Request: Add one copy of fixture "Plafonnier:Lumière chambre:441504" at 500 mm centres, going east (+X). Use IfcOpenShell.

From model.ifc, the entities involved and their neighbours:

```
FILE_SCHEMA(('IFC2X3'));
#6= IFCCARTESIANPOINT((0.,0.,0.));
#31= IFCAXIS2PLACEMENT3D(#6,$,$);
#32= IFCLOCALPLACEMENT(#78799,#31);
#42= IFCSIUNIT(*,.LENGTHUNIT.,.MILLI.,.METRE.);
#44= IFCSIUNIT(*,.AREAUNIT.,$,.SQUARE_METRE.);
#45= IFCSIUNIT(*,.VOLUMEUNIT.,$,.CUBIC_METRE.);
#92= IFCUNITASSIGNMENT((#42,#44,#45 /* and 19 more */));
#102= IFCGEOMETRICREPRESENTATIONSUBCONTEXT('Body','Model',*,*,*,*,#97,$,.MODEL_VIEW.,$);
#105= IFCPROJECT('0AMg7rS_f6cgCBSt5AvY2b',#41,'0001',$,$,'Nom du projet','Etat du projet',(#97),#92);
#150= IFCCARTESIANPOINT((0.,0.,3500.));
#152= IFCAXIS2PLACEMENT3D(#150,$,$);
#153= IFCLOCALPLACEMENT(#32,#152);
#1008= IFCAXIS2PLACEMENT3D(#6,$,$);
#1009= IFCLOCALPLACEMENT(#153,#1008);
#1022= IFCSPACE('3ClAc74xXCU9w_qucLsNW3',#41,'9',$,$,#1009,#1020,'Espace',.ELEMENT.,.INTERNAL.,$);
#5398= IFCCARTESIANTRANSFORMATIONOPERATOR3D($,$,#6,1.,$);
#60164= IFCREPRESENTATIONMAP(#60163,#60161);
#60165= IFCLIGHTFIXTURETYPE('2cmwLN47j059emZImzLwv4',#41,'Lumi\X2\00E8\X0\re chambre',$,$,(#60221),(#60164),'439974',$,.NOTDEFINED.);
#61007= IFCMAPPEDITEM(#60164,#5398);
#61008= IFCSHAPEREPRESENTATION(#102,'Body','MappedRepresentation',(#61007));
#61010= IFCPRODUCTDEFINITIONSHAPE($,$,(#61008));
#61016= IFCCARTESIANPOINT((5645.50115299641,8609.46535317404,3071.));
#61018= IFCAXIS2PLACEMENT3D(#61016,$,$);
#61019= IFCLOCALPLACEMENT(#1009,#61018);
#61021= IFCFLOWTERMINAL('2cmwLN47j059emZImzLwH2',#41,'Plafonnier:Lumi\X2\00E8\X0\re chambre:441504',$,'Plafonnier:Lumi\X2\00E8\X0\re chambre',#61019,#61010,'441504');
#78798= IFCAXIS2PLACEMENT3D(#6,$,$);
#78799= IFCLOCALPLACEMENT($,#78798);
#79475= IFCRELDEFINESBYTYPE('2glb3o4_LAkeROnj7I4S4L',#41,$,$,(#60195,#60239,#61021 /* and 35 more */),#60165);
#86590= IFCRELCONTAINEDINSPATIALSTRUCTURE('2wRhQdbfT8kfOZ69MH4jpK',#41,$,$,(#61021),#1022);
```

```python
import numpy as np
import ifcopenshell
import ifcopenshell.api.geometry
import ifcopenshell.api.root
import ifcopenshell.util.element
import ifcopenshell.util.placement

model = ifcopenshell.open("model.ifc")


def reuse_history(source, copy):
    """copy_class also copies each property set's owner history, people and application; keep the originals."""
    for rel in copy.IsDefinedBy:
        if rel.is_a("IfcRelDefinesByProperties") and (history := rel.RelatingPropertyDefinition.OwnerHistory):
            rel.RelatingPropertyDefinition.OwnerHistory = source.OwnerHistory
            ifcopenshell.util.element.remove_deep2(model, history)


source = model.by_guid("2cmwLN47j059emZImzLwH2")
base = ifcopenshell.util.placement.get_local_placement(source.ObjectPlacement)
step = np.array([1.0, 0.0, 0.0]) * 500.0

for i in range(1, 2):
    copy = ifcopenshell.api.root.copy_class(model, product=source)
    copy.Representation = ifcopenshell.util.element.copy_deep(
        model, source.Representation, exclude=["IfcGeometricRepresentationContext", "IfcRepresentationMap"]
    )
    copy.Name = "Plafonnier:Lumière chambre"
    copy.Tag = None
    reuse_history(source, copy)
    matrix = base.copy()
    matrix[:3, 3] += i * step
    print("added at", matrix[:3, 3].round(3) + 0.0)
    ifcopenshell.api.geometry.edit_object_placement(model, product=copy, matrix=matrix, is_si=False)

model.write("model_edited.ifc")
```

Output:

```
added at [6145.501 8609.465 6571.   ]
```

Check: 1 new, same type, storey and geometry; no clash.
